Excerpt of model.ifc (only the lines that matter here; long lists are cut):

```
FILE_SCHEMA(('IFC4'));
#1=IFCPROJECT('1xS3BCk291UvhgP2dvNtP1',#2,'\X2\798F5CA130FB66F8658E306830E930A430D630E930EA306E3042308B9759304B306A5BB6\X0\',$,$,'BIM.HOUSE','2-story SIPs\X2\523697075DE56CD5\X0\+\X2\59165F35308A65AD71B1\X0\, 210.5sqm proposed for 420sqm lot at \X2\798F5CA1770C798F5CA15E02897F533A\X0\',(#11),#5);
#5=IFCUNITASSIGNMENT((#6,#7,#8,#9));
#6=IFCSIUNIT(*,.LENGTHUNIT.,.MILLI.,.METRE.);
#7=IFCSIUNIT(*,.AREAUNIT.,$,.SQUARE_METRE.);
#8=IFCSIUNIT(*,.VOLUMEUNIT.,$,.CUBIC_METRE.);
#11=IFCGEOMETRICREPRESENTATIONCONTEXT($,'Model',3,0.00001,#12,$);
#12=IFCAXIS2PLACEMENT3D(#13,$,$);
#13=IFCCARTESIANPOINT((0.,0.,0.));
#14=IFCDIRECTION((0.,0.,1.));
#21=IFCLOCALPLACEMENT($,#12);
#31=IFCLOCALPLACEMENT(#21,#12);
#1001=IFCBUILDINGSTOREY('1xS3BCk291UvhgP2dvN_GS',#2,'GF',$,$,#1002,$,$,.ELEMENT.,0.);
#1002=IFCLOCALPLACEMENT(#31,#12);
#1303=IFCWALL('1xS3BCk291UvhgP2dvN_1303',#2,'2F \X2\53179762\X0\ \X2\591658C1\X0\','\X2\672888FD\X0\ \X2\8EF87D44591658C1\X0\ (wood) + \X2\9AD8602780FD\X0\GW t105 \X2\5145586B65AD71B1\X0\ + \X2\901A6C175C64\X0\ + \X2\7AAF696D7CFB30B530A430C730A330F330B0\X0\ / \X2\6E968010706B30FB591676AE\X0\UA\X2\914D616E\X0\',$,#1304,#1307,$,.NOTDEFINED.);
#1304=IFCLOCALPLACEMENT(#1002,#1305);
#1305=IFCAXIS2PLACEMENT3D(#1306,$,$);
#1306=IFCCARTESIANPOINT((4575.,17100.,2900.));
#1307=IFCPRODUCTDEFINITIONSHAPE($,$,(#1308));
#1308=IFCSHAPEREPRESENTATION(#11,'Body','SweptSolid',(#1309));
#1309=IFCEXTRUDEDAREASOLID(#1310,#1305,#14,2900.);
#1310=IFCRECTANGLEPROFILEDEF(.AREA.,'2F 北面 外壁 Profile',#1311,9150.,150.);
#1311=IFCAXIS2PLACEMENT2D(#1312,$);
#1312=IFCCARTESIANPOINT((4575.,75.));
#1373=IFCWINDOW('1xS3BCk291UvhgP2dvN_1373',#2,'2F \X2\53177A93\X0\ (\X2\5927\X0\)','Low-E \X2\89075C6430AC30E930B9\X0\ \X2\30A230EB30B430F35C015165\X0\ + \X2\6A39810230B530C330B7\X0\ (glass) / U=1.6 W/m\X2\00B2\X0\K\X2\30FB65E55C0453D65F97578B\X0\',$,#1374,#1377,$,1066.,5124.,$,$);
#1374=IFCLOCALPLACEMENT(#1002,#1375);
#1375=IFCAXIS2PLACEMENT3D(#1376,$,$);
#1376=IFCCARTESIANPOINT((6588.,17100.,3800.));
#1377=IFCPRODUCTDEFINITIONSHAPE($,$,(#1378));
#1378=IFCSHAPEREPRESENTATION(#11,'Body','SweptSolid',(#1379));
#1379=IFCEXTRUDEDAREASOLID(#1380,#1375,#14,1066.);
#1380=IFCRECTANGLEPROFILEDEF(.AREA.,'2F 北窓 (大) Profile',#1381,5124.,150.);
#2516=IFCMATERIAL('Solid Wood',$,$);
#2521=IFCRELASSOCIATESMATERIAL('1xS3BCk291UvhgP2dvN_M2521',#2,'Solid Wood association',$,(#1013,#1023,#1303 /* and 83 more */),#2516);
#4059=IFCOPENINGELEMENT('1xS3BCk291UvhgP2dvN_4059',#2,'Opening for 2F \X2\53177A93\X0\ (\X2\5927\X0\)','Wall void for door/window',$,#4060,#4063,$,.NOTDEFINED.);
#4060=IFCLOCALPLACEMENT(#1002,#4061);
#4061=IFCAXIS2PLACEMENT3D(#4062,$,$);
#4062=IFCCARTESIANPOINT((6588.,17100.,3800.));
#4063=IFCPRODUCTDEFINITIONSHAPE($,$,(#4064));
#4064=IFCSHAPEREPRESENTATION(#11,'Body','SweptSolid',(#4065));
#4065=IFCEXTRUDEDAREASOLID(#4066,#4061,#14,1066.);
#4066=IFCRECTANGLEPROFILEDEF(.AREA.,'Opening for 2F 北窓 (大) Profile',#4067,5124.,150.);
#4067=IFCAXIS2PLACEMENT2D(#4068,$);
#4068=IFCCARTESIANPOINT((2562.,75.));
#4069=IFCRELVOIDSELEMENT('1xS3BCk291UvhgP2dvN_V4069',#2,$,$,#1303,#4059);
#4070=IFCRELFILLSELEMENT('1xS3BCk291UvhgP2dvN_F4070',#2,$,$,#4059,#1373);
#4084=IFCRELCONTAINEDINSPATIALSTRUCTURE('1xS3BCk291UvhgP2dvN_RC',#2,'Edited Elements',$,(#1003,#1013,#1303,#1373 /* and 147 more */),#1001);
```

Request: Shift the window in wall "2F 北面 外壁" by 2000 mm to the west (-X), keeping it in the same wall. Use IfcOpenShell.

```python
import ifcopenshell
import ifcopenshell.api.geometry
import ifcopenshell.util.placement

model = ifcopenshell.open("model.ifc")

window = model.by_guid("1xS3BCk291UvhgP2dvN_1373")
opening = window.FillsVoids[0].RelatingOpeningElement
wall = opening.VoidsElements[0].RelatingBuildingElement

wall_matrix = ifcopenshell.util.placement.get_local_placement(wall.ObjectPlacement)
shift = wall_matrix[:3, 0] * -2000.0
before = ifcopenshell.util.placement.get_local_placement(window.ObjectPlacement)[:3, 3].copy()

# The window is not placed relative to its opening, so move both.
for product in (opening, window):
    matrix = ifcopenshell.util.placement.get_local_placement(product.ObjectPlacement)
    matrix[:3, 3] += shift
    ifcopenshell.api.geometry.edit_object_placement(model, product=product, matrix=matrix, is_si=False)

after = ifcopenshell.util.placement.get_local_placement(window.ObjectPlacement)[:3, 3]
print("window moved by", (after - before).round(3) + 0.0)

model.write("model_rev.ifc")
```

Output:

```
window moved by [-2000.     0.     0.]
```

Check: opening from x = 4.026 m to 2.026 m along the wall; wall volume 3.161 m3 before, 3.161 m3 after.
